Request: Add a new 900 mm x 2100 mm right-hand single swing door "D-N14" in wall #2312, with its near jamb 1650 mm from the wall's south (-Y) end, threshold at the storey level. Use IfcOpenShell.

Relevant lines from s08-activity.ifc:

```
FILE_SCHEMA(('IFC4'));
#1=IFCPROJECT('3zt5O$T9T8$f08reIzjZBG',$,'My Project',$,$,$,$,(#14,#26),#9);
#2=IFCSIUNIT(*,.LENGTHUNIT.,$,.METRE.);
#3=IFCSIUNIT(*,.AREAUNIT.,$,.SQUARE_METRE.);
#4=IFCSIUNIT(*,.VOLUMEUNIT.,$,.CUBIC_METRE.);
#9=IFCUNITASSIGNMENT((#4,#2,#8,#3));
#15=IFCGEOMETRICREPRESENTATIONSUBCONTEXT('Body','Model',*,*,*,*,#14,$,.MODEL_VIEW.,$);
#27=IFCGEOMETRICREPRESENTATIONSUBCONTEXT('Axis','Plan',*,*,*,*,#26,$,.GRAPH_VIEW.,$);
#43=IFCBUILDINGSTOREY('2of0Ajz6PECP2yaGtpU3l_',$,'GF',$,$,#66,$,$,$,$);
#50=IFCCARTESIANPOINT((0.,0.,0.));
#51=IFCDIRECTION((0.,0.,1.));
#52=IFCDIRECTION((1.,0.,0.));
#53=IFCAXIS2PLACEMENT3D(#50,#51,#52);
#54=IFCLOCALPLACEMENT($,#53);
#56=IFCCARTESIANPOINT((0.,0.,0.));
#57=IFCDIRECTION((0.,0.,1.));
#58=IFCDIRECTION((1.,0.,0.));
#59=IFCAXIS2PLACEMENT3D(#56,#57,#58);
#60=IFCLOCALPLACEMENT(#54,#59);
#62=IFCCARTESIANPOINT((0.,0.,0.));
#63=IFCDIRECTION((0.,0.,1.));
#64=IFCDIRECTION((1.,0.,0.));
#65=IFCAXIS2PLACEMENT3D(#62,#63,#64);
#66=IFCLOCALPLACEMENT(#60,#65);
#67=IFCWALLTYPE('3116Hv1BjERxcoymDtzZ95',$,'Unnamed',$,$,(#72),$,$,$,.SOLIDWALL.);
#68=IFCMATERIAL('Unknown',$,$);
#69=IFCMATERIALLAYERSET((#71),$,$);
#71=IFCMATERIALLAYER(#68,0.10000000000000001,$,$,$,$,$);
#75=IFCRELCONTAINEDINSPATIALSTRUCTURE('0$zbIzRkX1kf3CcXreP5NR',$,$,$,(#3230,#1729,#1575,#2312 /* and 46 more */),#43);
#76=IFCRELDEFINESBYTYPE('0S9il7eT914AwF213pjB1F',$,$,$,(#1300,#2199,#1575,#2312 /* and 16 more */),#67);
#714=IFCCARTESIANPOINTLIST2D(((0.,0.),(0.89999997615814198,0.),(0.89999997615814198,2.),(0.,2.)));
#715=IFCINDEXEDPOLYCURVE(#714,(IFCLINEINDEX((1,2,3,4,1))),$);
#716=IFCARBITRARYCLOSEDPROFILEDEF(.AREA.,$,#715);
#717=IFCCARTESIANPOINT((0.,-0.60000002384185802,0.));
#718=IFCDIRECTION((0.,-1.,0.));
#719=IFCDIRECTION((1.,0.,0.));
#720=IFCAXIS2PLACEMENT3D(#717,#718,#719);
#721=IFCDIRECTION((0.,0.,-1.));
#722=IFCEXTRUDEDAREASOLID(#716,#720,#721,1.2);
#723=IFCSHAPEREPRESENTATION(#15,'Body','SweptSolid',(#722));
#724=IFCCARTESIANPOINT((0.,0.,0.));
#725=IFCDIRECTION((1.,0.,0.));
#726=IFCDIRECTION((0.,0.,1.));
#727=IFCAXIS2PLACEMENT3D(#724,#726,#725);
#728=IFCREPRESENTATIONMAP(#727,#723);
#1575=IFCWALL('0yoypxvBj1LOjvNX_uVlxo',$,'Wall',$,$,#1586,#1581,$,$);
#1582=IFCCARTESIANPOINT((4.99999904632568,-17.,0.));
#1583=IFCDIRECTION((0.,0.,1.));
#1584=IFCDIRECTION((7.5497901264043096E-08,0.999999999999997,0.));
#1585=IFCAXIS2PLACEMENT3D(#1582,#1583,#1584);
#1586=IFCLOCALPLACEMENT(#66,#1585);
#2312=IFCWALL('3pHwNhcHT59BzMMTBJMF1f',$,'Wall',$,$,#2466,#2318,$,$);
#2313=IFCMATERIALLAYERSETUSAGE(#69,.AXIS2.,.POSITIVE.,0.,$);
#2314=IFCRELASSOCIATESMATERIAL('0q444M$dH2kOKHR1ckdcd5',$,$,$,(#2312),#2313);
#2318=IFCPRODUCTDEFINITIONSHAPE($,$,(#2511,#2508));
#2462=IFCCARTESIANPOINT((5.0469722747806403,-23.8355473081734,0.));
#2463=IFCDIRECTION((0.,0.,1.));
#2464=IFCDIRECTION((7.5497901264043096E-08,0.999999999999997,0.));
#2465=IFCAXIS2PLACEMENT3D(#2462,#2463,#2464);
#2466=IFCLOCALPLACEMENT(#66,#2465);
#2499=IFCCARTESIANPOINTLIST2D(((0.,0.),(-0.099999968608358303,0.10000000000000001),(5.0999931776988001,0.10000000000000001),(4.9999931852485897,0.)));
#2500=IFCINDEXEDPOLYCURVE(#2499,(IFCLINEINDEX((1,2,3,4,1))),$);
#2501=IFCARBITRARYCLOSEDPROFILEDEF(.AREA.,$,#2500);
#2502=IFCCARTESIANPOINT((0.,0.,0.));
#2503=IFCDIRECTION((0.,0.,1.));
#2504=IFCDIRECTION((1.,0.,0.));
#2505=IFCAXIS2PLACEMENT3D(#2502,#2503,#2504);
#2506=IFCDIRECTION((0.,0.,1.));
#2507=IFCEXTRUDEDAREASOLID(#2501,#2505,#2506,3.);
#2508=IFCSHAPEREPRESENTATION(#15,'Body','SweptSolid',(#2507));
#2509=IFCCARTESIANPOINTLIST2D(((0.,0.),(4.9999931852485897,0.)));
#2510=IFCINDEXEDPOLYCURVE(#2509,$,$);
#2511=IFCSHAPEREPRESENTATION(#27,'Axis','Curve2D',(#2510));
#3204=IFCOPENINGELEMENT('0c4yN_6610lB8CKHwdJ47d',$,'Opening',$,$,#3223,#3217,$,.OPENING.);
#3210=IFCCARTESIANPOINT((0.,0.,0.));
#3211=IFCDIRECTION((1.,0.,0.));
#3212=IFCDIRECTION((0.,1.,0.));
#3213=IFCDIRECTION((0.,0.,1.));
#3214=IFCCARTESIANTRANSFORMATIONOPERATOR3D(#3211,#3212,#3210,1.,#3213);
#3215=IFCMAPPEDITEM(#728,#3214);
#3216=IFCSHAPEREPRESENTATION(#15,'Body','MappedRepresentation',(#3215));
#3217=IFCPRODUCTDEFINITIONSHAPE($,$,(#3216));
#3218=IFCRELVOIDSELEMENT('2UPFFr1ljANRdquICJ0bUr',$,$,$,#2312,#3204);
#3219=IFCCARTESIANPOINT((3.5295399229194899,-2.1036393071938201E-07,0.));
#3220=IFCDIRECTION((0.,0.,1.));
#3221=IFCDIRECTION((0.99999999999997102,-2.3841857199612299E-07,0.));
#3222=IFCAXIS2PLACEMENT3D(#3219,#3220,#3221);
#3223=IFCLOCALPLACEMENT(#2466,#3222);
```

```python
import numpy as np
import ifcopenshell
import ifcopenshell.api.feature
import ifcopenshell.api.geometry
import ifcopenshell.api.root
import ifcopenshell.api.spatial
import ifcopenshell.geom
import ifcopenshell.util.element
import ifcopenshell.util.placement
import ifcopenshell.util.representation
import ifcopenshell.util.shape
import ifcopenshell.util.unit

model = ifcopenshell.open("s08-activity.ifc")
unit_scale = ifcopenshell.util.unit.calculate_unit_scale(model)
settings = ifcopenshell.geom.settings()


def volume(element):
    """Net volume in cubic metres, openings subtracted."""
    shape = ifcopenshell.geom.create_shape(settings, element)
    return ifcopenshell.util.shape.get_volume(shape.geometry)


wall = model.by_id(2312)
storey = ifcopenshell.util.element.get_container(wall, ifc_class="IfcBuildingStorey")
context = ifcopenshell.util.representation.get_context(model, "Model", "Body", "MODEL_VIEW")
before = volume(wall)

width, height, from_end, sill = 0.9, 2.1, 1.65, 0.0  # metres

# The wall runs along its own X axis, and the end named is its -X end.
wall_shape = ifcopenshell.geom.create_shape(settings, wall)
x, y, z = ifcopenshell.util.shape.get_vertices(wall_shape.geometry).T
start = x.min() + from_end
face, thickness = float(y.min()), float(y.max() - y.min())
wall_matrix = ifcopenshell.util.placement.get_local_placement(wall.ObjectPlacement)
level = ifcopenshell.util.placement.get_local_placement(storey.ObjectPlacement)[2, 3]


def in_wall(x, y):
    """Placement at x, y metres in the wall's axes, at sill height."""
    matrix = wall_matrix.copy()
    matrix[:, 3] = wall_matrix @ np.array([x / unit_scale, y / unit_scale, 0.0, 1.0])
    matrix[2, 3] = level + sill / unit_scale
    return matrix


# Opening: a box that overshoots both wall faces by 50 mm.
opening = ifcopenshell.api.root.create_entity(model, ifc_class="IfcOpeningElement", predefined_type="OPENING")
box = ifcopenshell.api.geometry.add_wall_representation(
    model, context=context, length=width, height=height, thickness=thickness + 0.1
)
ifcopenshell.api.geometry.assign_representation(model, product=opening, representation=box)
ifcopenshell.api.geometry.edit_object_placement(model, product=opening, matrix=in_wall(start, face - 0.05), is_si=False)
ifcopenshell.api.feature.add_feature(model, feature=opening, element=wall)

door = ifcopenshell.api.root.create_entity(model, ifc_class="IfcDoor", name="D-N14", predefined_type="DOOR")
door.OverallWidth, door.OverallHeight = width / unit_scale, height / unit_scale
door.OperationType = "SINGLE_SWING_RIGHT"
body = ifcopenshell.api.geometry.add_door_representation(
    model,
    context=context,
    overall_width=door.OverallWidth,
    overall_height=door.OverallHeight,
    operation_type="SINGLE_SWING_RIGHT",
    lining_properties={"LiningDepth": thickness / unit_scale, "ThresholdDepth": thickness / unit_scale},
)
ifcopenshell.api.geometry.assign_representation(model, product=door, representation=body)
ifcopenshell.api.spatial.assign_container(model, products=[door], relating_structure=storey)
ifcopenshell.api.feature.add_filling(model, opening=opening, element=door)

# The lining spans the wall, so the door starts at the wall face.
ifcopenshell.api.geometry.edit_object_placement(model, product=door, matrix=in_wall(start, face), is_si=False)

after = volume(wall)

print(f"wall volume {before:.3f} -> {after:.3f} m3")

model.write("s08-activity_edited.ifc")
```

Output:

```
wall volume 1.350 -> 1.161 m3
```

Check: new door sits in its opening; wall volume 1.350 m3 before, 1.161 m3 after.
